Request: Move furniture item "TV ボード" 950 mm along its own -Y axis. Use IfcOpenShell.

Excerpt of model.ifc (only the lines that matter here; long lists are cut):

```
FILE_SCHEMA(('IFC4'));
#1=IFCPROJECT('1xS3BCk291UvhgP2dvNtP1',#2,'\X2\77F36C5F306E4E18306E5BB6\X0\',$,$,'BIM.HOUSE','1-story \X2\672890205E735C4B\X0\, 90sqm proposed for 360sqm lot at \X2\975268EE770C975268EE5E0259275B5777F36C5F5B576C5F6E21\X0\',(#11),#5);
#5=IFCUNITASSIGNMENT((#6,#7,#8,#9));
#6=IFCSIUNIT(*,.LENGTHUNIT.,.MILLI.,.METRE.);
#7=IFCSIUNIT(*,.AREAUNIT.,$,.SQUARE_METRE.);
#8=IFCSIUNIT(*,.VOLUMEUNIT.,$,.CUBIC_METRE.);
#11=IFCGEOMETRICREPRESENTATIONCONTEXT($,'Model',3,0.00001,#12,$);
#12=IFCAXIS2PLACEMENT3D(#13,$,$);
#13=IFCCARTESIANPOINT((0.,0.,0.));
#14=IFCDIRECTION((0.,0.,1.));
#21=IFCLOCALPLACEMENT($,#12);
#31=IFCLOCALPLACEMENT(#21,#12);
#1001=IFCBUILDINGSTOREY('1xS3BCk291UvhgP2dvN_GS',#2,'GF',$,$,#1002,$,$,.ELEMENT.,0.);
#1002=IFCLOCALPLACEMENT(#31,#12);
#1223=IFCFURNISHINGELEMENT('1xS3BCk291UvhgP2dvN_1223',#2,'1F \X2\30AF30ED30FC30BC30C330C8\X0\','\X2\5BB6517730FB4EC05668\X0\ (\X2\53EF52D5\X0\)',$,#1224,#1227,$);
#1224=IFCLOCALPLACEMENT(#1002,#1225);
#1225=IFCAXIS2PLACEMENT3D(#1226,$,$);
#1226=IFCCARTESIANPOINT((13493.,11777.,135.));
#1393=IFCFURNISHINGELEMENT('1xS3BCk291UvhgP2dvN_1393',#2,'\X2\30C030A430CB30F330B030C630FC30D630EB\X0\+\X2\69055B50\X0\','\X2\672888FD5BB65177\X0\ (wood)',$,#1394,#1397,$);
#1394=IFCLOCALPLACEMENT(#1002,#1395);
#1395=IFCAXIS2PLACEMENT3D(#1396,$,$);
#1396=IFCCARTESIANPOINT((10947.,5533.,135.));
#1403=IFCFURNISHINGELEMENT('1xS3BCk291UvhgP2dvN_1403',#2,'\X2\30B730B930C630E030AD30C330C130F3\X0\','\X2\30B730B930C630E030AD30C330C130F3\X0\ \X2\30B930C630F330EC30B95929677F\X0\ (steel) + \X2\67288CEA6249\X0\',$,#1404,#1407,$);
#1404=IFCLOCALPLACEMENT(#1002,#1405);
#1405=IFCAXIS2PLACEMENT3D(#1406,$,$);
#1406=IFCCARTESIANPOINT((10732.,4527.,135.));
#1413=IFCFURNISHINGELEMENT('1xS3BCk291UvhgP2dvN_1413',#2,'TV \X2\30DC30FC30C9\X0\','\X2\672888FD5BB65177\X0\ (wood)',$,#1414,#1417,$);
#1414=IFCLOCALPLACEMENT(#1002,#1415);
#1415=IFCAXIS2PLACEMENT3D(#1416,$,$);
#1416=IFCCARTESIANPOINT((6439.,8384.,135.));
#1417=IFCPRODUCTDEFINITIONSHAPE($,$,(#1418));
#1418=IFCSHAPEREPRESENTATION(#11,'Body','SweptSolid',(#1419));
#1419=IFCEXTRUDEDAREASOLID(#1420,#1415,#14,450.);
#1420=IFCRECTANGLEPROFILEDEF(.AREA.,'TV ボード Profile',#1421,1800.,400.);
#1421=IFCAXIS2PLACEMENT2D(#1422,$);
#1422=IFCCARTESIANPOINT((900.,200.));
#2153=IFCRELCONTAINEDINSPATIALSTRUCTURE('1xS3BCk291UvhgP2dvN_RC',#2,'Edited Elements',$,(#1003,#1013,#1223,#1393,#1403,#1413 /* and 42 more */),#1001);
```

```python
import ifcopenshell
import ifcopenshell.api.geometry
import ifcopenshell.util.placement

model = ifcopenshell.open("model.ifc")

item = model.by_guid("1xS3BCk291UvhgP2dvN_1413")
matrix = ifcopenshell.util.placement.get_local_placement(item.ObjectPlacement)
matrix[:3, 3] -= matrix[:3, 1] * 950.0
ifcopenshell.api.geometry.edit_object_placement(model, product=item, matrix=matrix, is_si=False)

print(ifcopenshell.util.placement.get_local_placement(item.ObjectPlacement).round(3) + 0.0)

model.write("model_updated.ifc")
```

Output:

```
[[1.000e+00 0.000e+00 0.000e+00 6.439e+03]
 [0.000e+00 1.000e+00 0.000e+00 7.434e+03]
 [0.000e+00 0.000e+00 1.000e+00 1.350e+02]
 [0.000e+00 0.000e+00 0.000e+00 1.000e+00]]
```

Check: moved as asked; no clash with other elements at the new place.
